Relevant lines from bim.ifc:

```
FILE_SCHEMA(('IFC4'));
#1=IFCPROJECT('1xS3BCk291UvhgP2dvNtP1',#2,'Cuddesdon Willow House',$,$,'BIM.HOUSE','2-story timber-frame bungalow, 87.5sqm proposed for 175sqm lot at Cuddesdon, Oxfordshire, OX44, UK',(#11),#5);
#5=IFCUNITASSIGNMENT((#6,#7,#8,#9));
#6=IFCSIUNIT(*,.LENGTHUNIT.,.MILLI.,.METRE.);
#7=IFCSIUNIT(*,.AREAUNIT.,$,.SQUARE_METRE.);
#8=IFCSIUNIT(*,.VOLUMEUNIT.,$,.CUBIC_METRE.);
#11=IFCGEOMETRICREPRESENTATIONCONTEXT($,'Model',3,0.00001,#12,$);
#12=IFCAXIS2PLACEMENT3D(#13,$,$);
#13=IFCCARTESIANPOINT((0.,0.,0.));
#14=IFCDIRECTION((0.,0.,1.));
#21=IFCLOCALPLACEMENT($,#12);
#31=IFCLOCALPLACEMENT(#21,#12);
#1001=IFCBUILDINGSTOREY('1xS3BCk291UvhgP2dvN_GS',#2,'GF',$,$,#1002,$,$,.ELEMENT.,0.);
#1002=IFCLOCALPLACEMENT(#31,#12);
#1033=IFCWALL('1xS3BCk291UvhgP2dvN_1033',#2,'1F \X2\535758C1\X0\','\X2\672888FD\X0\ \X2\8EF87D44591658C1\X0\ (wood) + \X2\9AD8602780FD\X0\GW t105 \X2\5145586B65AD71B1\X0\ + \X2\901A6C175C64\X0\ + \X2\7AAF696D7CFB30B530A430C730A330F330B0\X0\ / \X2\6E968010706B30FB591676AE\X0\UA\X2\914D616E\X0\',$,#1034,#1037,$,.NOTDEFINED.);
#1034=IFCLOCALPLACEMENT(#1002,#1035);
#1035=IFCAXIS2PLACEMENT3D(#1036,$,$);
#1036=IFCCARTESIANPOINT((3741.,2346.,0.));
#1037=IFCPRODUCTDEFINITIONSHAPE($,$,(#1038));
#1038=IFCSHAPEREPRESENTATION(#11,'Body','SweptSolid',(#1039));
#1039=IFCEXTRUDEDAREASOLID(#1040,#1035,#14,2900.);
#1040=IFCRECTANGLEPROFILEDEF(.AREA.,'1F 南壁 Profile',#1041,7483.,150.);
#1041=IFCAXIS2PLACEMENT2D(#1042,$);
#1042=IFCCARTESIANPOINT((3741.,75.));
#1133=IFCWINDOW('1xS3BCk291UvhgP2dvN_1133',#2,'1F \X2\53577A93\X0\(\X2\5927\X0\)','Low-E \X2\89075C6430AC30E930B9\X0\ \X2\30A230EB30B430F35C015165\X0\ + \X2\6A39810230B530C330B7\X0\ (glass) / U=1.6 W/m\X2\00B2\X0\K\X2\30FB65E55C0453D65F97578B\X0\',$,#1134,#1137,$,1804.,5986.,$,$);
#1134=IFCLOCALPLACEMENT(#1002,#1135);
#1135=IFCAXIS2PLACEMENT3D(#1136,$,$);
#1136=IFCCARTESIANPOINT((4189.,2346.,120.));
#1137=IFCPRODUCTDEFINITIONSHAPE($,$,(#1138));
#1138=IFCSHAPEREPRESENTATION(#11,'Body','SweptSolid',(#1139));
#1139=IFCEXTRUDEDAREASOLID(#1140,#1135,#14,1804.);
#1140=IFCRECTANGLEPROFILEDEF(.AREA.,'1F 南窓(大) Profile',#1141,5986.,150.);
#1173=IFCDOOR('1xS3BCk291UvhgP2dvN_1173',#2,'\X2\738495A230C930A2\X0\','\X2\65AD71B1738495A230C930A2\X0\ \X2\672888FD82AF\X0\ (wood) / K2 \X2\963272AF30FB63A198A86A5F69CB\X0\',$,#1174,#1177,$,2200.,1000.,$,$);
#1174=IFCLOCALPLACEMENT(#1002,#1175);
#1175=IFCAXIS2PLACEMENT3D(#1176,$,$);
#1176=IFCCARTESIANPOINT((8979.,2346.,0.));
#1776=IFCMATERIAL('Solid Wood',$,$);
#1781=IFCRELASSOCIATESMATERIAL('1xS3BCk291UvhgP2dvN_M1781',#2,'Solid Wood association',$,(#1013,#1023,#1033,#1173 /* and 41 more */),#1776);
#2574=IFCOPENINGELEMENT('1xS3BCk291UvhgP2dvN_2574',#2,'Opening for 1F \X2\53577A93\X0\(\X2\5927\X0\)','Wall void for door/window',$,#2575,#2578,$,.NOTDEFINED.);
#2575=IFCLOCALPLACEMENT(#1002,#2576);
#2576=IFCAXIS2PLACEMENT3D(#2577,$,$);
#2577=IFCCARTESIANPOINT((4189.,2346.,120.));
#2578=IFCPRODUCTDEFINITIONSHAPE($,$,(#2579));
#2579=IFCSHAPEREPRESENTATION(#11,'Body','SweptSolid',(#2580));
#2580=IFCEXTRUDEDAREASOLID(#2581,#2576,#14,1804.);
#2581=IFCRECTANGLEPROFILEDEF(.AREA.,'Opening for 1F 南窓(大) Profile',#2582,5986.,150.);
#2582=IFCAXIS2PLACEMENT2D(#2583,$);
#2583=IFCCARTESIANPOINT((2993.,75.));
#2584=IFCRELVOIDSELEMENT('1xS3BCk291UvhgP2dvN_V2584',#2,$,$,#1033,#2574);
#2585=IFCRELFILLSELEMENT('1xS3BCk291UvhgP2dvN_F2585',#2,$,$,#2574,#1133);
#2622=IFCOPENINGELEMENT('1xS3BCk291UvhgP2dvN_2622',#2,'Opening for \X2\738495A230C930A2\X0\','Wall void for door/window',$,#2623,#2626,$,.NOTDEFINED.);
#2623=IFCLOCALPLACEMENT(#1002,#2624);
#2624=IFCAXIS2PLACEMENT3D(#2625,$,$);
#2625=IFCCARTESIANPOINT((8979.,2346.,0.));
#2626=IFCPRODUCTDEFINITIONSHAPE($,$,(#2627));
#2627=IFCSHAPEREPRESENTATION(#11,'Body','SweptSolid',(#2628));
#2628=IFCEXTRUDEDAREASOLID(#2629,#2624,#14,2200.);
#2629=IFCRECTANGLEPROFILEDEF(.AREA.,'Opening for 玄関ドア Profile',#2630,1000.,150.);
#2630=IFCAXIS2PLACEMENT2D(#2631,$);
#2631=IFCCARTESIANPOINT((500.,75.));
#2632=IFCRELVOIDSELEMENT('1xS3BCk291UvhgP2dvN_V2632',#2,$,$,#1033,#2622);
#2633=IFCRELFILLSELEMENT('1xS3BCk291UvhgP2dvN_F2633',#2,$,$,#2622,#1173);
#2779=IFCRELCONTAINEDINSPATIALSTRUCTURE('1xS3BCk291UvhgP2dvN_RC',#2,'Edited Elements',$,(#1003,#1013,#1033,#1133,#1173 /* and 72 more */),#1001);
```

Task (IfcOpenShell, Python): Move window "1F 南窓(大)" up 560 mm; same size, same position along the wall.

```python
import numpy as np
import ifcopenshell
import ifcopenshell.api.geometry
import ifcopenshell.util.placement
import ifcopenshell.util.unit

model = ifcopenshell.open("bim.ifc")
unit_scale = ifcopenshell.util.unit.calculate_unit_scale(model)

window = model.by_guid("1xS3BCk291UvhgP2dvN_1133")
opening = window.FillsVoids[0].RelatingOpeningElement
dz = 0.56 / unit_scale

shift = np.array([0.0, 0.0, dz])
# The window is not placed relative to its opening, so move both.
for product in (opening, window):
    matrix = ifcopenshell.util.placement.get_local_placement(product.ObjectPlacement)
    matrix[:3, 3] += shift
    ifcopenshell.api.geometry.edit_object_placement(model, product=product, matrix=matrix, is_si=False)

print(f"moved by {dz * unit_scale:+.3f} m")

model.write("bim_edited.ifc")
```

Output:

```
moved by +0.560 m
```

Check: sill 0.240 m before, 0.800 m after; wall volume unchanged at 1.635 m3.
